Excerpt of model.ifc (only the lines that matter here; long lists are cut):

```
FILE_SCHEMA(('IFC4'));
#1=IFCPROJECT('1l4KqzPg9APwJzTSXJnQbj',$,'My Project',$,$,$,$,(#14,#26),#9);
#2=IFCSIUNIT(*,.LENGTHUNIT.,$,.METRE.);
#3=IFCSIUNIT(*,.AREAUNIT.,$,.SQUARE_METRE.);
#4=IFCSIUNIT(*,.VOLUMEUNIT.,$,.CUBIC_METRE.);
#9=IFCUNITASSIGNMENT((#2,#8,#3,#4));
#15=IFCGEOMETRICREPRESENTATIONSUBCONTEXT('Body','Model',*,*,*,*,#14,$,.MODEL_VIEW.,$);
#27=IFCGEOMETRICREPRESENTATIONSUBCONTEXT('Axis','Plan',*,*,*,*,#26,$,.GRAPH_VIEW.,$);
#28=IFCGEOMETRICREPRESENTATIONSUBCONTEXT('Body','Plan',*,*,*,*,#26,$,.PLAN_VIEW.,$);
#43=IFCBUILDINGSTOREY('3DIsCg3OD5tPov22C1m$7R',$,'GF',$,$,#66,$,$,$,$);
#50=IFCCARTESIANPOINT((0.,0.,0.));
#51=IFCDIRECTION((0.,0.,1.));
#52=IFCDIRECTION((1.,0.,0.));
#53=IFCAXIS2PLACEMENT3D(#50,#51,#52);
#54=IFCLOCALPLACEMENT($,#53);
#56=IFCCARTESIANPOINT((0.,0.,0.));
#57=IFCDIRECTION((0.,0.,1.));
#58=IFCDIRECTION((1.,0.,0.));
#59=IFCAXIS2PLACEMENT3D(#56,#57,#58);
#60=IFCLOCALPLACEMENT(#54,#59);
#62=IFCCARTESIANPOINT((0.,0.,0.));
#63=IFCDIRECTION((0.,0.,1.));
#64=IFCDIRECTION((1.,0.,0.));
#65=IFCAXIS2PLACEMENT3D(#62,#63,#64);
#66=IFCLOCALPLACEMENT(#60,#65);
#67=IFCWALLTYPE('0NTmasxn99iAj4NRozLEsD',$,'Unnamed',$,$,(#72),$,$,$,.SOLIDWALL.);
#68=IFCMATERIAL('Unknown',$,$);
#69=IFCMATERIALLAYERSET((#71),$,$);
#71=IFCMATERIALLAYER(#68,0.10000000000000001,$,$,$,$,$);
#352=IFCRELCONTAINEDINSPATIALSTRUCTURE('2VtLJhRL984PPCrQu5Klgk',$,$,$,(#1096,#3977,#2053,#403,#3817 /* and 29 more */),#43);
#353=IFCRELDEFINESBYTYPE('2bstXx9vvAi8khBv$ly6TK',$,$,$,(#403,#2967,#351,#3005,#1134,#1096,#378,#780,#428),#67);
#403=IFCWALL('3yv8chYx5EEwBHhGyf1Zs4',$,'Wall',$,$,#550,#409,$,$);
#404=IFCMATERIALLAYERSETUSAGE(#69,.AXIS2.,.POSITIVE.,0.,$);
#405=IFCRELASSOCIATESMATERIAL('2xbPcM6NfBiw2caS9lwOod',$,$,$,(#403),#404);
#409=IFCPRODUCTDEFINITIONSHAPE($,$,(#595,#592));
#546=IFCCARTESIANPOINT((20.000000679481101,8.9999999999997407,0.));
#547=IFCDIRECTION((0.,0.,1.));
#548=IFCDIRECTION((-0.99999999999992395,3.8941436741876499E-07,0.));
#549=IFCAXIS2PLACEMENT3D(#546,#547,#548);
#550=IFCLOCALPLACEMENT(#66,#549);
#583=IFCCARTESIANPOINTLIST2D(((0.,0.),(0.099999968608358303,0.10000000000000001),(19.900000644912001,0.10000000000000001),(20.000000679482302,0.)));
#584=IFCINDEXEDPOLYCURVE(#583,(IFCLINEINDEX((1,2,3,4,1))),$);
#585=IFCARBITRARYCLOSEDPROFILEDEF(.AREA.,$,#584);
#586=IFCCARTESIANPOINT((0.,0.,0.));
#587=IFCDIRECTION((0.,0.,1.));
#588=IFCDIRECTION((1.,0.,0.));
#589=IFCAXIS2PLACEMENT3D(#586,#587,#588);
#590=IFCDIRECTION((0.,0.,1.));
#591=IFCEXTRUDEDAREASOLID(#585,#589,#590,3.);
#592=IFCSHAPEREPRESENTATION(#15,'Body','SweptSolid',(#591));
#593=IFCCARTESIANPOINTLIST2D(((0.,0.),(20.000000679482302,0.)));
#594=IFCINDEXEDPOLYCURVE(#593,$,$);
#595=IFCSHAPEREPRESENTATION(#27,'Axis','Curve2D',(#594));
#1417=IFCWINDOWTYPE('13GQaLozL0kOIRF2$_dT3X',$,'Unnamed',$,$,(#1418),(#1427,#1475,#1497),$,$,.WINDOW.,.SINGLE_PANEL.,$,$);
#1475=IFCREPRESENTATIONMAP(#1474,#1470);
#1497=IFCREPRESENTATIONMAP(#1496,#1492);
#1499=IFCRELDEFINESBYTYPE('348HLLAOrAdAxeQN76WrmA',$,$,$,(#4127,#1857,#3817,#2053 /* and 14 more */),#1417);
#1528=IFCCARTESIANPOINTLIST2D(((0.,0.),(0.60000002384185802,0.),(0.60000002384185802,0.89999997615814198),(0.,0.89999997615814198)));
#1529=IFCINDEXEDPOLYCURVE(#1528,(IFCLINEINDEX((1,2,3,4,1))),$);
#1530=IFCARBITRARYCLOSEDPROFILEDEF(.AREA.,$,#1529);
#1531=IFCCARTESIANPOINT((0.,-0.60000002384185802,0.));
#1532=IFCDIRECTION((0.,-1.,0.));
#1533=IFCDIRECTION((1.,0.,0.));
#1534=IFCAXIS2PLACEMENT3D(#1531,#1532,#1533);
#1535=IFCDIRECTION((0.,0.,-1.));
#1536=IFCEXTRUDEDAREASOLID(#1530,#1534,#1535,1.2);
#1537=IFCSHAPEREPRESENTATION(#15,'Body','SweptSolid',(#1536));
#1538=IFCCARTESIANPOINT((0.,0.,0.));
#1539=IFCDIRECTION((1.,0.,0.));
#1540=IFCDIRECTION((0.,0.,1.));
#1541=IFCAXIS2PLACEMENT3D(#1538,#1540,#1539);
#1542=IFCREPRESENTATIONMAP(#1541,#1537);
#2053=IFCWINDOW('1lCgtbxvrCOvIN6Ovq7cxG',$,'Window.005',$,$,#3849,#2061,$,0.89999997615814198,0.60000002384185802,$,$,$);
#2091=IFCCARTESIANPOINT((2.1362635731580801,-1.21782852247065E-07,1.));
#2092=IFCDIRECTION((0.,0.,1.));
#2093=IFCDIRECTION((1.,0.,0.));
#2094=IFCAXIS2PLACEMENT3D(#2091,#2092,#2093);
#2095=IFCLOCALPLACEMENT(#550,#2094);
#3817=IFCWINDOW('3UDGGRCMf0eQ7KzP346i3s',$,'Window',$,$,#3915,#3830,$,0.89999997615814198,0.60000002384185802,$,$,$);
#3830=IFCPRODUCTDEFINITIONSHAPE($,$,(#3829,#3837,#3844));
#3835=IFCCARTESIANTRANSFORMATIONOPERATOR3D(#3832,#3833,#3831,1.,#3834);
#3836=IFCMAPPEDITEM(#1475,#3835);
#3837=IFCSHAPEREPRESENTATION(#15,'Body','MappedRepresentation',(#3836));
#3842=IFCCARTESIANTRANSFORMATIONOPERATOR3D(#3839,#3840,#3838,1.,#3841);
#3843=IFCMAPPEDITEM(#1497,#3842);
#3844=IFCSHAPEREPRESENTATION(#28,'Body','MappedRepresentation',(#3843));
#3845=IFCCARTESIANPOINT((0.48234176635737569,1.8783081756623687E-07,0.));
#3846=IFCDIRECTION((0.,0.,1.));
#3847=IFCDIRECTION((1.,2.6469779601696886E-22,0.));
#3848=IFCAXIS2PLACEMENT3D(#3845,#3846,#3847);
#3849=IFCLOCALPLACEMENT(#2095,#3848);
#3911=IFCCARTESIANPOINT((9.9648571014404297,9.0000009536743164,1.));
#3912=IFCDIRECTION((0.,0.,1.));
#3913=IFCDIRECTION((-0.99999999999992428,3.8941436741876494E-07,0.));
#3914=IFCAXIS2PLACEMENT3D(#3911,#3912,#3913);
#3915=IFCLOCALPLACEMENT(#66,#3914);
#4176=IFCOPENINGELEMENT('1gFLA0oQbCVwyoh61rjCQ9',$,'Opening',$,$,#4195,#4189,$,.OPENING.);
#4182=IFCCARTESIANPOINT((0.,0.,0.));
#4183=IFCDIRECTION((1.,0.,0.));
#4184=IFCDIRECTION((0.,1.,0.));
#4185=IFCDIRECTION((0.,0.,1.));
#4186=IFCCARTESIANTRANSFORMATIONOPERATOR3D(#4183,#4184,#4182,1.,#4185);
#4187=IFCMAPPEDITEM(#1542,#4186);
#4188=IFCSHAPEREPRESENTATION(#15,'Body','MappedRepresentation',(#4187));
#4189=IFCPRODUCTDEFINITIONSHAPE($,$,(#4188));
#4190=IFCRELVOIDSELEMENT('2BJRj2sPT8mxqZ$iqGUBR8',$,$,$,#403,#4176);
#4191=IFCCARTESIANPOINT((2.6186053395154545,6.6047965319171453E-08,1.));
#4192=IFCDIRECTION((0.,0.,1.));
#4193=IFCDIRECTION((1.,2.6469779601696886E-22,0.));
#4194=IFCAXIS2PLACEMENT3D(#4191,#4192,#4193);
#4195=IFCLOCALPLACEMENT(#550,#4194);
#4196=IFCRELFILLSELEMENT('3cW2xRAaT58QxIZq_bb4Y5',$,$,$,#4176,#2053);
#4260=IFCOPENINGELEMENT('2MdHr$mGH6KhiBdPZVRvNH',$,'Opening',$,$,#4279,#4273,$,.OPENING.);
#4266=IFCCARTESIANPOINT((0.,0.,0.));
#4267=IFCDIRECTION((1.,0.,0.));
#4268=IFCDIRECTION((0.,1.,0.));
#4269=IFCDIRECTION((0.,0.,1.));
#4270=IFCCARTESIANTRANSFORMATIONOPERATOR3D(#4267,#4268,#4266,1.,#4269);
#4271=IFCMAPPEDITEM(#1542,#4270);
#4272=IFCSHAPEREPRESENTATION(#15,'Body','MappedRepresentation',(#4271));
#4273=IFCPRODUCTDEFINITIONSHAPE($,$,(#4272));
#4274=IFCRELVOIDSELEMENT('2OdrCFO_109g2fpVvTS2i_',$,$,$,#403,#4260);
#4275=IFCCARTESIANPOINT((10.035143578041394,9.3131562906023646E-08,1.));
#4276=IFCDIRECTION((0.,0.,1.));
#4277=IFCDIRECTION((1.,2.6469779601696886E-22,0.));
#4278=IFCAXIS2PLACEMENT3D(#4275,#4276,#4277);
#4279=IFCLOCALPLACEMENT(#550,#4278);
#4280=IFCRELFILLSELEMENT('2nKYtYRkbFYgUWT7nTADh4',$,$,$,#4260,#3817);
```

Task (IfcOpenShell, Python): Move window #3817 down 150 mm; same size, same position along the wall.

```python
import numpy as np
import ifcopenshell
import ifcopenshell.api.geometry
import ifcopenshell.util.placement
import ifcopenshell.util.unit

model = ifcopenshell.open("model.ifc")
unit_scale = ifcopenshell.util.unit.calculate_unit_scale(model)

window = model.by_guid("3UDGGRCMf0eQ7KzP346i3s")
opening = window.FillsVoids[0].RelatingOpeningElement
dz = -0.15 / unit_scale

shift = np.array([0.0, 0.0, dz])
# The window is not placed relative to its opening, so move both.
for product in (opening, window):
    matrix = ifcopenshell.util.placement.get_local_placement(product.ObjectPlacement)
    matrix[:3, 3] += shift
    ifcopenshell.api.geometry.edit_object_placement(model, product=product, matrix=matrix, is_si=False)

print(f"moved by {dz * unit_scale:+.3f} m")

model.write("model_edited.ifc")
```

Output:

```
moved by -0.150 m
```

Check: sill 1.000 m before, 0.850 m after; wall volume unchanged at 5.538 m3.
